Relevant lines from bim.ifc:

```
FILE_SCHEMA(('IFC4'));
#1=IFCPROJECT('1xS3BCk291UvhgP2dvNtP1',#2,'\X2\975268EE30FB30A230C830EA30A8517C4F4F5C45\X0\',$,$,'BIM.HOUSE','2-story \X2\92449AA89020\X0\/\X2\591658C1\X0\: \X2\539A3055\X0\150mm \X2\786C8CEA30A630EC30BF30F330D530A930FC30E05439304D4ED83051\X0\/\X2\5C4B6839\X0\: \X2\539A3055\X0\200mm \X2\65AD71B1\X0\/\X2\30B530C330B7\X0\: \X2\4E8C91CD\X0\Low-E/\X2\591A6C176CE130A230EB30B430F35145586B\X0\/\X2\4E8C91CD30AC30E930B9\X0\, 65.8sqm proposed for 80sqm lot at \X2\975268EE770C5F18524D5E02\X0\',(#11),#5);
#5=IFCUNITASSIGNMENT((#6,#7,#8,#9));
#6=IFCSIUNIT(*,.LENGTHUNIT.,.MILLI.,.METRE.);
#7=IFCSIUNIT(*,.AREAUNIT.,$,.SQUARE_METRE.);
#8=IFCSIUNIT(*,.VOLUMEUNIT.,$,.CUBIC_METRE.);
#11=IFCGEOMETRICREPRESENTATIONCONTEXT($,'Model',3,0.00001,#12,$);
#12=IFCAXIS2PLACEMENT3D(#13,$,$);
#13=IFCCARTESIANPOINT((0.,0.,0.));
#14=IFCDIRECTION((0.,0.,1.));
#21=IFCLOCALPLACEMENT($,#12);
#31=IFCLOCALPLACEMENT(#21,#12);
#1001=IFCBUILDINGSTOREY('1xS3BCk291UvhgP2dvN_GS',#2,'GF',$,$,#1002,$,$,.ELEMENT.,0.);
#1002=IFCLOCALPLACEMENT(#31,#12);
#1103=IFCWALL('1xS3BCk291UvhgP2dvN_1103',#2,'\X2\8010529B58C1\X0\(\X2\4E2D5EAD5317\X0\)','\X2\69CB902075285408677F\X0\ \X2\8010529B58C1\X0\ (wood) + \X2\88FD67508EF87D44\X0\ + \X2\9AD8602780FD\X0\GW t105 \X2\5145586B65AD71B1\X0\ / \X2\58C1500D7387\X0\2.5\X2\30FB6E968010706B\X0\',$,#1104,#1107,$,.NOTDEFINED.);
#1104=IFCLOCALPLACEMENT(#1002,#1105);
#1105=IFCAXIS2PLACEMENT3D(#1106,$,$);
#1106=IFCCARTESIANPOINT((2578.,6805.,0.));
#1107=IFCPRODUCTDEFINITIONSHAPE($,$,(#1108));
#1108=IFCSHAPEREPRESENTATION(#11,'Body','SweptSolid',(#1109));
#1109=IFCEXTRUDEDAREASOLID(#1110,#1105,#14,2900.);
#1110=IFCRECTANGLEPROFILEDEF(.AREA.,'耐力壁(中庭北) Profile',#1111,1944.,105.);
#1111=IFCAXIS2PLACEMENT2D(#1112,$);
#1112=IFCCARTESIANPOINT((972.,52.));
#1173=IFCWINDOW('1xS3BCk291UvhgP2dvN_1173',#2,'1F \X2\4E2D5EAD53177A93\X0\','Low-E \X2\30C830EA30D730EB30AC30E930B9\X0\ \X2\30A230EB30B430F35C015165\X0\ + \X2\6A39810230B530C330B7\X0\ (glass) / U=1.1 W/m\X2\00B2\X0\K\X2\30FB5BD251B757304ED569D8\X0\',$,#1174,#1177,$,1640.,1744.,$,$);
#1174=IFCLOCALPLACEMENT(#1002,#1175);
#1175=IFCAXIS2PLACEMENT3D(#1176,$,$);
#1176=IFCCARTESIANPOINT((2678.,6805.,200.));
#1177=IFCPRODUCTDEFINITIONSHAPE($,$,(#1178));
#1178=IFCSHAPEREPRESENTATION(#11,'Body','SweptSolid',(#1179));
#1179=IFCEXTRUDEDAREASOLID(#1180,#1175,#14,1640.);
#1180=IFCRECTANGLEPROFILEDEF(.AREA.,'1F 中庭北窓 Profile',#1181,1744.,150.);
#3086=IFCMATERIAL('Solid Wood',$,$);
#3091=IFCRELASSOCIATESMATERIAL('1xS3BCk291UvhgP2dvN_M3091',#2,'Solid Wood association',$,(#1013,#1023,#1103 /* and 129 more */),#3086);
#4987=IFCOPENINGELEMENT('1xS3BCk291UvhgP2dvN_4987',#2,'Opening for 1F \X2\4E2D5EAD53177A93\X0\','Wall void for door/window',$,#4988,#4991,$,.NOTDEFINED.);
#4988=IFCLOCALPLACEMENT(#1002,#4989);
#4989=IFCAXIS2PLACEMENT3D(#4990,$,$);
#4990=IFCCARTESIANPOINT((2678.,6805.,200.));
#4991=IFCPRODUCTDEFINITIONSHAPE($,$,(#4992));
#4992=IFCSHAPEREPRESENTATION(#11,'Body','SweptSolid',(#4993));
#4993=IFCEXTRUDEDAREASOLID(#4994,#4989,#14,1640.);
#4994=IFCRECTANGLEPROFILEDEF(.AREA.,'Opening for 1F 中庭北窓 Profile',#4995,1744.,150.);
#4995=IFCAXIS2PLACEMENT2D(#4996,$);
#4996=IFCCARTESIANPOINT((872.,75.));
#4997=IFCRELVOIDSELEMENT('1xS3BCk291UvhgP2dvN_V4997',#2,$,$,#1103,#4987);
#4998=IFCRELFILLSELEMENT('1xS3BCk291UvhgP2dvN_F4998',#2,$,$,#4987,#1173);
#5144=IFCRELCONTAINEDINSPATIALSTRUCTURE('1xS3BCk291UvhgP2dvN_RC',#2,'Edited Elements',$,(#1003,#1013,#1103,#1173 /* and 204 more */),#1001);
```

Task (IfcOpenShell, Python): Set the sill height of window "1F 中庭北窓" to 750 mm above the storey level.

```python
import numpy as np
import ifcopenshell
import ifcopenshell.api.geometry
import ifcopenshell.geom
import ifcopenshell.util.element
import ifcopenshell.util.placement
import ifcopenshell.util.shape
import ifcopenshell.util.unit

model = ifcopenshell.open("bim.ifc")
unit_scale = ifcopenshell.util.unit.calculate_unit_scale(model)

window = model.by_id(1173)
opening = window.FillsVoids[0].RelatingOpeningElement
storey = ifcopenshell.util.element.get_container(window, ifc_class="IfcBuildingStorey")
level = ifcopenshell.util.placement.get_local_placement(storey.ObjectPlacement)[2, 3]

# The opening's origin need not be at the sill, so measure its lowest point.
shape = ifcopenshell.geom.create_shape(ifcopenshell.geom.settings(), opening)
bottom = ifcopenshell.util.shape.get_shape_bottom_elevation(shape, shape.geometry) / unit_scale
dz = level + 0.75 / unit_scale - bottom

shift = np.array([0.0, 0.0, dz])
# The window is not placed relative to its opening, so move both.
for product in (opening, window):
    matrix = ifcopenshell.util.placement.get_local_placement(product.ObjectPlacement)
    matrix[:3, 3] += shift
    ifcopenshell.api.geometry.edit_object_placement(model, product=product, matrix=matrix, is_si=False)

print(f"moved by {dz * unit_scale:+.3f} m")

model.write("bim-out.ifc")
```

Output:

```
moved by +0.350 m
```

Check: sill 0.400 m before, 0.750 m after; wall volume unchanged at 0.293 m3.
